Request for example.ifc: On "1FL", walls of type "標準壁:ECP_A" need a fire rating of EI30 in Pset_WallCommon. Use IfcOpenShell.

First a look at what the model holds.

```python
import ifcopenshell
import ifcopenshell.util.element

model = ifcopenshell.open("example.ifc")
print(model.schema)
storey = next(s for s in model.by_type("IfcBuildingStorey") if s.Name == "1FL")
walls = [e for e in ifcopenshell.util.element.get_decomposition(storey) if e.is_a("IfcWall")]
seen = {}
for e in walls:
    element_type = ifcopenshell.util.element.get_type(e)
    key = (element_type.Name if element_type != e and element_type else None, ifcopenshell.util.element.get_pset(e, "Pset_WallCommon", "FireRating"))
    seen[key] = seen.get(key, 0) + 1
for (name, value), count in sorted(seen.items(), key=str):
    print(count, "x", name, "|", value)
```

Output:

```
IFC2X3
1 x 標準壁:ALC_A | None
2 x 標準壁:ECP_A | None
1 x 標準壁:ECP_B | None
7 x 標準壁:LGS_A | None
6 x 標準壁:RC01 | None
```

```python
import ifcopenshell
import ifcopenshell.api.pset
import ifcopenshell.util.element

model = ifcopenshell.open("example.ifc")

storey = next(s for s in model.by_type("IfcBuildingStorey") if s.Name == "1FL")
walls = [e for e in ifcopenshell.util.element.get_decomposition(storey) if e.is_a("IfcWall")]

count = 0
for e in walls:
    element_type = ifcopenshell.util.element.get_type(e)
    if element_type in (None, e) or element_type.Name != "標準壁:ECP_A":
        continue
    # add_pset returns the element's existing set when there is one.
    pset = ifcopenshell.api.pset.add_pset(model, product=e, name="Pset_WallCommon")
    ifcopenshell.api.pset.edit_pset(model, pset=pset, properties={"FireRating": "EI30"})
    count += 1

print(count, "walls updated")

model.write("example_rev.ifc")
```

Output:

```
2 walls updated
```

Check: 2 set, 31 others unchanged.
